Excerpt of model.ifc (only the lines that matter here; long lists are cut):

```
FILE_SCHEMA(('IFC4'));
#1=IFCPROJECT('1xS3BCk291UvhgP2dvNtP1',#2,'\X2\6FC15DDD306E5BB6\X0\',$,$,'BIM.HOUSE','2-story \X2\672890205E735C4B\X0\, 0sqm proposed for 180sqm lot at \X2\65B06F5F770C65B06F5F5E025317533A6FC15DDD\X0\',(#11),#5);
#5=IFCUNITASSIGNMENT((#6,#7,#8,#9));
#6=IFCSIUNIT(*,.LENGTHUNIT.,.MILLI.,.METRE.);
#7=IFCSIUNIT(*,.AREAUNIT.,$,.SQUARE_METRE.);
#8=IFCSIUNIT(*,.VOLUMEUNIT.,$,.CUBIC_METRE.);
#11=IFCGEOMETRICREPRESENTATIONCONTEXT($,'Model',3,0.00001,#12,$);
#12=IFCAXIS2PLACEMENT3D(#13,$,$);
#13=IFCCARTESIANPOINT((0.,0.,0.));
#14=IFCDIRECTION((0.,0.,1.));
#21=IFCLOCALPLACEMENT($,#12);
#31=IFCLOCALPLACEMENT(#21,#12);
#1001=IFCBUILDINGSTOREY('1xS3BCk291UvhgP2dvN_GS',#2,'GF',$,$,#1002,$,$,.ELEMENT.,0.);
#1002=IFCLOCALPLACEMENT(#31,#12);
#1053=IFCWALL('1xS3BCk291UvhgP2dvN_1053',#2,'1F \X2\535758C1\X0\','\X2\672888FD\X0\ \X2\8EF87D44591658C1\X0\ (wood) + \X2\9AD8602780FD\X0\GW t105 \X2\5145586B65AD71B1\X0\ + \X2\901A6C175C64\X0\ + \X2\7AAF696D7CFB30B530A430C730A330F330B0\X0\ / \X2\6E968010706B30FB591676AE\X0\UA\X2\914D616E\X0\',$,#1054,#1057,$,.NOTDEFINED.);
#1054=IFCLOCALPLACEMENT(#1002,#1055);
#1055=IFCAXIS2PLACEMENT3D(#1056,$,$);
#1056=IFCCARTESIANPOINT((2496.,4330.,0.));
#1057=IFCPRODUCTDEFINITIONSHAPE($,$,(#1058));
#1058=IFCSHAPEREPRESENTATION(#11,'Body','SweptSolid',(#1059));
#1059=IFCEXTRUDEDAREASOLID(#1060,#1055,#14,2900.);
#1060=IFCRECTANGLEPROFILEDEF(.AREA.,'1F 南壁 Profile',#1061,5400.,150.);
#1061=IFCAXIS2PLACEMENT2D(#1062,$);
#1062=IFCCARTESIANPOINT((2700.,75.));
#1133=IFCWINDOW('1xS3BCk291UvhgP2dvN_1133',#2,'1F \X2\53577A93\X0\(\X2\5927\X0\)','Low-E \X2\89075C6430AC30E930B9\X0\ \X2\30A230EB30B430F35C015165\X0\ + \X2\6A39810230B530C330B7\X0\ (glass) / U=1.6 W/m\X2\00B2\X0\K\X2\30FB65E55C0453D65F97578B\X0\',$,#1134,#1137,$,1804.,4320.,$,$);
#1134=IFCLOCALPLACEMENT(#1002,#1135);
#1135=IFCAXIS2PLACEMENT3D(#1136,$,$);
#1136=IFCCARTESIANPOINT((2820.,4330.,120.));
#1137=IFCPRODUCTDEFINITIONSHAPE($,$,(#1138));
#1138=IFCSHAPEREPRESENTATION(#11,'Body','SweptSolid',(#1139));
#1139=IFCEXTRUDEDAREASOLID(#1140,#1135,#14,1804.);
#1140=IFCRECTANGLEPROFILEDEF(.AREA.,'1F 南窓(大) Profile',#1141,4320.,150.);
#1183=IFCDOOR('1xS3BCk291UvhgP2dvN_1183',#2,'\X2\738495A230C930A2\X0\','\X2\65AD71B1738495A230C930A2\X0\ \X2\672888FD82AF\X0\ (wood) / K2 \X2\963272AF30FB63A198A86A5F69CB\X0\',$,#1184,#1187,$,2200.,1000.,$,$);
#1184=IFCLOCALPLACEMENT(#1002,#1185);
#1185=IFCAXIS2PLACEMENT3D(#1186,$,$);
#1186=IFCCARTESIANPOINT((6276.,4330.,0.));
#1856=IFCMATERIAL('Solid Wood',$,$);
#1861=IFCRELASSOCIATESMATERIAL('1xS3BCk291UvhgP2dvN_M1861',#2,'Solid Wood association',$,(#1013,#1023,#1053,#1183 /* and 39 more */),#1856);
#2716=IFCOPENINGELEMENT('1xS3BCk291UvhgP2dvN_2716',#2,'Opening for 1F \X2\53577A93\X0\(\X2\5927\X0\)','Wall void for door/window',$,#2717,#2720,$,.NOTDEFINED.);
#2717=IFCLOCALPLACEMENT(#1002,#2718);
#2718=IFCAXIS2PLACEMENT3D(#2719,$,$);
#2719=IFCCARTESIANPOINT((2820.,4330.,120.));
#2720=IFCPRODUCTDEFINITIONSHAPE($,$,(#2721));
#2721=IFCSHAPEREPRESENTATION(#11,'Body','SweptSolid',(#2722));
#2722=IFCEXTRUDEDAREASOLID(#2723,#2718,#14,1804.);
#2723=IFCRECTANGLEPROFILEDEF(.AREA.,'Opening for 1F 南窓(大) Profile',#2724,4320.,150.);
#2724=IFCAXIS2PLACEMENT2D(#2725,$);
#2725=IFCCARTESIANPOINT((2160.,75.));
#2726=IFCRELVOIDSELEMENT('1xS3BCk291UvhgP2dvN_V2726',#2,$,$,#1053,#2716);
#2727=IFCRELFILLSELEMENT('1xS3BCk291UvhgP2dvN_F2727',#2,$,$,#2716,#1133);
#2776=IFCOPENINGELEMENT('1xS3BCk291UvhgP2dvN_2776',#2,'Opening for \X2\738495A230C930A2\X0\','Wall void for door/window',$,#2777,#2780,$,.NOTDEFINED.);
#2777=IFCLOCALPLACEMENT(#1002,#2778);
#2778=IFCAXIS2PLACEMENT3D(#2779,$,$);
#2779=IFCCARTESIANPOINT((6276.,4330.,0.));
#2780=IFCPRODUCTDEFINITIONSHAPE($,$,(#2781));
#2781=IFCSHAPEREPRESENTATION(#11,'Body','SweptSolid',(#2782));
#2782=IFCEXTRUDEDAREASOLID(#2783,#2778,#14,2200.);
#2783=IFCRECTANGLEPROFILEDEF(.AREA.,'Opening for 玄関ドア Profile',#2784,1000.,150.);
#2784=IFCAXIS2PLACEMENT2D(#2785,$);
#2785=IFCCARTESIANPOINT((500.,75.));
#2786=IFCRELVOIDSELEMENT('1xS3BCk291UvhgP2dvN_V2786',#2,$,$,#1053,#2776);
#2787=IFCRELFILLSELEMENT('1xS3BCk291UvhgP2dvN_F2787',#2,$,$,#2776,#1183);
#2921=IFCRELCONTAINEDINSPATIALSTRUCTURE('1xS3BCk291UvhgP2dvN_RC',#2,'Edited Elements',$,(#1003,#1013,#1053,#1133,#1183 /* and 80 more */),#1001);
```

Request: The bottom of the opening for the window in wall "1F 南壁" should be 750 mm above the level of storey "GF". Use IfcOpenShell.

```python
import numpy as np
import ifcopenshell
import ifcopenshell.api.geometry
import ifcopenshell.geom
import ifcopenshell.util.element
import ifcopenshell.util.placement
import ifcopenshell.util.shape
import ifcopenshell.util.unit

model = ifcopenshell.open("model.ifc")
unit_scale = ifcopenshell.util.unit.calculate_unit_scale(model)

window = model.by_guid("1xS3BCk291UvhgP2dvN_1133")
opening = window.FillsVoids[0].RelatingOpeningElement
storey = ifcopenshell.util.element.get_container(window, ifc_class="IfcBuildingStorey")
level = ifcopenshell.util.placement.get_local_placement(storey.ObjectPlacement)[2, 3]

# The opening's origin need not be at the sill, so measure its lowest point.
shape = ifcopenshell.geom.create_shape(ifcopenshell.geom.settings(), opening)
bottom = ifcopenshell.util.shape.get_shape_bottom_elevation(shape, shape.geometry) / unit_scale
dz = level + 750.0 - bottom

shift = np.array([0.0, 0.0, dz])
# The window is not placed relative to its opening, so move both.
for product in (opening, window):
    matrix = ifcopenshell.util.placement.get_local_placement(product.ObjectPlacement)
    matrix[:3, 3] += shift
    ifcopenshell.api.geometry.edit_object_placement(model, product=product, matrix=matrix, is_si=False)

print(f"moved by {dz * unit_scale:+.3f} m")

model.write("model_v2.ifc")
```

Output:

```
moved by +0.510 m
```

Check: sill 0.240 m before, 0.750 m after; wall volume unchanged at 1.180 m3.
